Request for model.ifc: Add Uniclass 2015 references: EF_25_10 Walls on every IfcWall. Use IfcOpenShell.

First a look at what the model holds.

```python
import ifcopenshell

model = ifcopenshell.open("model.ifc")
print(model.schema)
print("classifications:", [c.Name for c in model.by_type("IfcClassification")])
for ifc_class in ("IfcDoor", "IfcRoof", "IfcStair", "IfcWall", "IfcWindow"):
    print(ifc_class, len(model.by_type(ifc_class)))
```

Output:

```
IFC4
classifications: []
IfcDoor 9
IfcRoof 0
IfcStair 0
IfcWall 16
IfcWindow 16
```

```python
import ifcopenshell
import ifcopenshell.api.classification

model = ifcopenshell.open("model.ifc")

system = ifcopenshell.api.classification.add_classification(model, classification="Uniclass 2015")

codes = {
    "IfcWall": ("EF_25_10", "Walls"),
}
for ifc_class, (code, name) in codes.items():
    products = model.by_type(ifc_class)
    ifcopenshell.api.classification.add_reference(
        model, products=products, classification=system, identification=code, name=name
    )
    print(code, len(products))

model.write("model-out.ifc")
```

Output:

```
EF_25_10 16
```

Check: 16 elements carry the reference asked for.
